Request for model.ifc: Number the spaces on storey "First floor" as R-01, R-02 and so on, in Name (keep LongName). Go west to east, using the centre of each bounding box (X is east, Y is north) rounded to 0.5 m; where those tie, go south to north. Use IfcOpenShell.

First a look at what the model holds.

```python
import ifcopenshell
import ifcopenshell.util.element
import ifcopenshell.util.placement

model = ifcopenshell.open("model.ifc")
print(model.schema)
storey = next(s for s in model.by_type("IfcBuildingStorey") if s.Name == "First floor")
spaces = [e for e in ifcopenshell.util.element.get_decomposition(storey) if e.is_a("IfcSpace")]
for e in sorted(spaces, key=lambda e: e.id()):
    origin = ifcopenshell.util.placement.get_local_placement(e.ObjectPlacement)[:3, 3]
    print(e.id(), e.Name, e.LongName, origin.round(2) + 0.0, sep=" | ")
```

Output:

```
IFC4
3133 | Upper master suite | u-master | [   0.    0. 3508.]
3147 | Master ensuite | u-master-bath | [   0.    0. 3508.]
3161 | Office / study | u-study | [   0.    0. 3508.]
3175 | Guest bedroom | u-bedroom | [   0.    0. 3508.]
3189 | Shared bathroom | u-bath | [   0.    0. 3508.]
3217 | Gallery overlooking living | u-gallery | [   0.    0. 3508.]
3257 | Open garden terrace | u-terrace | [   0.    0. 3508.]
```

```python
import ifcopenshell
import ifcopenshell.geom
import ifcopenshell.util.element
import ifcopenshell.util.shape

model = ifcopenshell.open("model.ifc")
settings = ifcopenshell.geom.settings()
settings.set("use-world-coords", True)


def centre(element):
    shape = ifcopenshell.geom.create_shape(settings, element)
    return ifcopenshell.util.shape.get_bbox_centroid(shape.geometry)


storey = next(s for s in model.by_type("IfcBuildingStorey") if s.Name == "First floor")
spaces = [e for e in ifcopenshell.util.element.get_decomposition(storey) if e.is_a("IfcSpace")]

# Insertion points can sit at a corner or the storey origin, so sort by the geometry (in metres).
centres = {e: centre(e) for e in spaces}
spaces.sort(key=lambda e: (round(centres[e][0] / 0.5), centres[e][1]))

for i, e in enumerate(spaces, start=1):
    number = f"R-{i:02d}"
    e.Name = number
    print(e.id(), number)

model.write("model_updated.ifc")
```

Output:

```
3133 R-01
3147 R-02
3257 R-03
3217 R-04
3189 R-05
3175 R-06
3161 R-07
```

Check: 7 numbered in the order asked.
